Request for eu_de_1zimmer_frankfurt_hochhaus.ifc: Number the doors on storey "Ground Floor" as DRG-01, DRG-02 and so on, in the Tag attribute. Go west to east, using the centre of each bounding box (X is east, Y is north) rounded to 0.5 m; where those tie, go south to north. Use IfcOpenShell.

First a look at what the model holds.

```python
import ifcopenshell
import ifcopenshell.util.element
import ifcopenshell.util.placement

model = ifcopenshell.open("eu_de_1zimmer_frankfurt_hochhaus.ifc")
print(model.schema)
storey = next(s for s in model.by_type("IfcBuildingStorey") if s.Name == "Ground Floor")
doors = [e for e in ifcopenshell.util.element.get_decomposition(storey) if e.is_a("IfcDoor")]
for e in sorted(doors, key=lambda e: e.id()):
    origin = ifcopenshell.util.placement.get_local_placement(e.ObjectPlacement)[:3, 3]
    print(e.id(), e.Tag, e.Name, origin.round(2) + 0.0, sep=" | ")
```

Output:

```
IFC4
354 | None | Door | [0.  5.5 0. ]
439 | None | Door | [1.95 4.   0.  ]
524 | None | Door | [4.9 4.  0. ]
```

```python
import ifcopenshell
import ifcopenshell.geom
import ifcopenshell.util.element
import ifcopenshell.util.shape

model = ifcopenshell.open("eu_de_1zimmer_frankfurt_hochhaus.ifc")
settings = ifcopenshell.geom.settings()
settings.set("use-world-coords", True)


def centre(element):
    shape = ifcopenshell.geom.create_shape(settings, element)
    return ifcopenshell.util.shape.get_bbox_centroid(shape.geometry)


storey = next(s for s in model.by_type("IfcBuildingStorey") if s.Name == "Ground Floor")
doors = [e for e in ifcopenshell.util.element.get_decomposition(storey) if e.is_a("IfcDoor")]

# Insertion points can sit at a corner or the storey origin, so sort by the geometry (in metres).
centres = {e: centre(e) for e in doors}
doors.sort(key=lambda e: (round(centres[e][0] / 0.5), centres[e][1]))

for i, e in enumerate(doors, start=1):
    number = f"DRG-{i:02d}"
    e.Tag = number
    print(e.id(), number)

model.write("eu_de_1zimmer_frankfurt_hochhaus_v2.ifc")
```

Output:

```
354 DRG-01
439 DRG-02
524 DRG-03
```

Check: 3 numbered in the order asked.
